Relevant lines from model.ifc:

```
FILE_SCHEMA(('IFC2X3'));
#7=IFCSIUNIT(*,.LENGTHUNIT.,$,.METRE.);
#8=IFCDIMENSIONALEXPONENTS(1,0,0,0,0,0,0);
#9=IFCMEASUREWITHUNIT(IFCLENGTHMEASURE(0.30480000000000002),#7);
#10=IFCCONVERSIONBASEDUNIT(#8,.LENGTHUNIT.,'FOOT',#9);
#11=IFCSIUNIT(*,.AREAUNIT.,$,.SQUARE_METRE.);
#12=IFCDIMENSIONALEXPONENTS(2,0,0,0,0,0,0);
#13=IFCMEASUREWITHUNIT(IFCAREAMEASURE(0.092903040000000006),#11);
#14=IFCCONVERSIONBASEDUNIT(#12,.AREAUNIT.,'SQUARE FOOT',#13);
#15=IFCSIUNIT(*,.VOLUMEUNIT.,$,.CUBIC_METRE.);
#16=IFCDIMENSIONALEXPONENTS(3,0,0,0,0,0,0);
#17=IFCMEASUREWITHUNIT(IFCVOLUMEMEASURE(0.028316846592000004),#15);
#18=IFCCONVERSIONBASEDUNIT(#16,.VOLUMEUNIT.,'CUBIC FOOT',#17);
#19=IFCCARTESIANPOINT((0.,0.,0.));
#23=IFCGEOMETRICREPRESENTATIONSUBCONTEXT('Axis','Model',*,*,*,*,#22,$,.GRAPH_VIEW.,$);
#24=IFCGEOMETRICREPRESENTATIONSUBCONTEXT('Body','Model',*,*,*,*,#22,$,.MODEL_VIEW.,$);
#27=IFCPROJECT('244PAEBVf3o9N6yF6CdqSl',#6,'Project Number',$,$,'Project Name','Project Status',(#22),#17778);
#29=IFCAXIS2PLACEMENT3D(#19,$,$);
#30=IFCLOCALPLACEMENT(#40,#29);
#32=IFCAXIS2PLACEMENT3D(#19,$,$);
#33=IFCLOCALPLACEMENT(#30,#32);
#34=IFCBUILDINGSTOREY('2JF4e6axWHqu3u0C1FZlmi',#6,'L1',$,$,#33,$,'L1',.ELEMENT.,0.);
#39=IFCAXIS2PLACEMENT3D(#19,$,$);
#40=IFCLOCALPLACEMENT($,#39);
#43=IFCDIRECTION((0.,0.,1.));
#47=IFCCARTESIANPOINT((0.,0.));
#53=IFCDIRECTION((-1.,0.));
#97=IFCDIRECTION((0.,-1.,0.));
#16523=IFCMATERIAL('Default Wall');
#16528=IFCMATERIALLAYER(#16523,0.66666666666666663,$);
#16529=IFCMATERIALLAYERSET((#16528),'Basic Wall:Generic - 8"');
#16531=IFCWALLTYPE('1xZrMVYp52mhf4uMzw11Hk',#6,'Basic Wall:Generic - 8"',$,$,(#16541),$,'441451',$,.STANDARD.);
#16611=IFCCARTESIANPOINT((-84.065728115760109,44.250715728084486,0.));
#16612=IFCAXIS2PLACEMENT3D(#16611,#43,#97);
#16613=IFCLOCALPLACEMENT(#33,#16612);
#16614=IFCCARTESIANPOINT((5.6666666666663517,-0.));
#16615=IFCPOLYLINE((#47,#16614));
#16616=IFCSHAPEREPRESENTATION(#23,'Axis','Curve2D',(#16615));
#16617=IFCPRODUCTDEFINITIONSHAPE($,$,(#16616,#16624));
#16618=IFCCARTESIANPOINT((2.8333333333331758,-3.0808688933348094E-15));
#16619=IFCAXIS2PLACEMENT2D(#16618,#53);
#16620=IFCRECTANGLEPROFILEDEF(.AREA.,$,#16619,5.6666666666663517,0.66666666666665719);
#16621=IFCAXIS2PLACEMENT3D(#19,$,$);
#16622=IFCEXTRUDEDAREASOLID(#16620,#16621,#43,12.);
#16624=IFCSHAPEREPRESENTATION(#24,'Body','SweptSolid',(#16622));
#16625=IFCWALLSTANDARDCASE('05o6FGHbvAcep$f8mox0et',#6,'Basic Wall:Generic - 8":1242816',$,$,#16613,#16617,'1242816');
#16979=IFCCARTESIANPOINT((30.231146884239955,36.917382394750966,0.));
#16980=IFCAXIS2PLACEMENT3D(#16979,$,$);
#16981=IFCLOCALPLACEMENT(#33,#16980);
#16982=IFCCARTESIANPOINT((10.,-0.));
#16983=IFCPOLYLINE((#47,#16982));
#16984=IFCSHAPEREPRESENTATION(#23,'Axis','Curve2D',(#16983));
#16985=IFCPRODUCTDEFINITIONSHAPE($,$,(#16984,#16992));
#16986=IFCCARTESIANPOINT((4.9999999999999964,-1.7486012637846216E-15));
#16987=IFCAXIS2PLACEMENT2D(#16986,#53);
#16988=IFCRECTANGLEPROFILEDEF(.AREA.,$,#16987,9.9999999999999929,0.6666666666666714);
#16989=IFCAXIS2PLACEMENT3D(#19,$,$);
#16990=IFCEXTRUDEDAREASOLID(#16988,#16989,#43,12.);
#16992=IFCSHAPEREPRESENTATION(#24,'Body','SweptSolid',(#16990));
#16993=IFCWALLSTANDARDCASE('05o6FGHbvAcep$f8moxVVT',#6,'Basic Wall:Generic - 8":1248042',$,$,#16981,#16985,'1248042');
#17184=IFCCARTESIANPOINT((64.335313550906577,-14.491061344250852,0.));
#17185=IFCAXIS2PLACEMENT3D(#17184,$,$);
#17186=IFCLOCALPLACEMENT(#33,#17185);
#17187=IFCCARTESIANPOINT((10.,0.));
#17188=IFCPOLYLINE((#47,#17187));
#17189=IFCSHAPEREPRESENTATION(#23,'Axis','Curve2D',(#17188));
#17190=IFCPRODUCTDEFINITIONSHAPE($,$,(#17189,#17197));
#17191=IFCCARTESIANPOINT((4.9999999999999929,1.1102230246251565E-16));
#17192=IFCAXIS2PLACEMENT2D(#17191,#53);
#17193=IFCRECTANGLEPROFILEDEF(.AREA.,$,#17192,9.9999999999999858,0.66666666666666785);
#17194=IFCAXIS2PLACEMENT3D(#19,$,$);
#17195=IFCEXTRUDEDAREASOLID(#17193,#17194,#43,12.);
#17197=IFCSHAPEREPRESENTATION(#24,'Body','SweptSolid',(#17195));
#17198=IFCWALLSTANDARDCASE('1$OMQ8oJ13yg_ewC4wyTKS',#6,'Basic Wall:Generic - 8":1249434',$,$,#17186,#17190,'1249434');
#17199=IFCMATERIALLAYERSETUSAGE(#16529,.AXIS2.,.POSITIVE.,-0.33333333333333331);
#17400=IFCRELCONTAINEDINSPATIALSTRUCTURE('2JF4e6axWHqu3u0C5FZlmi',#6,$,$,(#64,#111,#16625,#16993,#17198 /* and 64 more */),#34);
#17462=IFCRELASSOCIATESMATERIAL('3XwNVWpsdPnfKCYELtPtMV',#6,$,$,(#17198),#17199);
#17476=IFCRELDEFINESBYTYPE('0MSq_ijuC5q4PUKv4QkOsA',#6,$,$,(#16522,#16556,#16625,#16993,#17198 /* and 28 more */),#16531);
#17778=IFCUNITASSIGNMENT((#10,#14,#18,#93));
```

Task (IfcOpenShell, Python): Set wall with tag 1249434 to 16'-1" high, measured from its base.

```python
import ifcopenshell
import ifcopenshell.geom
import ifcopenshell.util.representation
import ifcopenshell.util.shape
import ifcopenshell.util.unit

model = ifcopenshell.open("model.ifc")
unit_scale = ifcopenshell.util.unit.calculate_unit_scale(model)
settings = ifcopenshell.geom.settings()


def volume(element):
    """Net volume in cubic metres, openings subtracted."""
    shape = ifcopenshell.geom.create_shape(settings, element)
    return ifcopenshell.util.shape.get_volume(shape.geometry)


wall = model.by_id(17198)
before = volume(wall)

body = ifcopenshell.util.representation.get_representation(wall, "Model", "Body")
solid = body.Items[0]
old_height = solid.Depth
solid.Depth = 193 * 0.0254 / unit_scale
after = volume(wall)

print(f"height {old_height:g} -> {solid.Depth:g}, volume {before:.3f} -> {after:.3f} m3")

model.write("model-out.ifc")
```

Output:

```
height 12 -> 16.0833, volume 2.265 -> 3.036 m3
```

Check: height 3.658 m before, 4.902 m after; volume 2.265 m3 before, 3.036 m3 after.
